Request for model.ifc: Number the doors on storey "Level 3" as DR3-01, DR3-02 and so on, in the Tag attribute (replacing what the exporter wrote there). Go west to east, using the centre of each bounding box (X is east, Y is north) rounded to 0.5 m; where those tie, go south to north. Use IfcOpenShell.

First a look at what the model holds.

```python
import ifcopenshell
import ifcopenshell.util.element
import ifcopenshell.util.placement

model = ifcopenshell.open("model.ifc")
print(model.schema)
storey = next(s for s in model.by_type("IfcBuildingStorey") if s.Name == "Level 3")
doors = [e for e in ifcopenshell.util.element.get_decomposition(storey) if e.is_a("IfcDoor")]
for e in sorted(doors, key=lambda e: e.id()):
    origin = ifcopenshell.util.placement.get_local_placement(e.ObjectPlacement)[:3, 3]
    print(e.id(), e.Tag, e.Name, origin.round(2) + 0.0, sep=" | ")
```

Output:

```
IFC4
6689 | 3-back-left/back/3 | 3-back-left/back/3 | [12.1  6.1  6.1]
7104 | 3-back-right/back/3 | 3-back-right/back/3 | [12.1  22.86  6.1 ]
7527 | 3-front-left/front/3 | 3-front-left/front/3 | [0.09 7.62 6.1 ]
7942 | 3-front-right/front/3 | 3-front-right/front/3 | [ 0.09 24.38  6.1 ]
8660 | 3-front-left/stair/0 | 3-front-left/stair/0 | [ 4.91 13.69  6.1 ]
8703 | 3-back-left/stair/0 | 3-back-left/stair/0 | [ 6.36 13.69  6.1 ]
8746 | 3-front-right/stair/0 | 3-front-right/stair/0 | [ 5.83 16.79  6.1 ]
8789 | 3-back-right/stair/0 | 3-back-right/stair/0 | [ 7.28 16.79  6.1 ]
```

```python
import ifcopenshell
import ifcopenshell.geom
import ifcopenshell.util.element
import ifcopenshell.util.shape

model = ifcopenshell.open("model.ifc")
settings = ifcopenshell.geom.settings()
settings.set("use-world-coords", True)


def centre(element):
    shape = ifcopenshell.geom.create_shape(settings, element)
    return ifcopenshell.util.shape.get_bbox_centroid(shape.geometry)


storey = next(s for s in model.by_type("IfcBuildingStorey") if s.Name == "Level 3")
doors = [e for e in ifcopenshell.util.element.get_decomposition(storey) if e.is_a("IfcDoor")]

# Insertion points can sit at a corner or the storey origin, so sort by the geometry (in metres).
centres = {e: centre(e) for e in doors}
doors.sort(key=lambda e: (round(centres[e][0] / 0.5), centres[e][1]))

for i, e in enumerate(doors, start=1):
    number = f"DR3-{i:02d}"
    e.Tag = number
    print(e.id(), number)

model.write("model_v2.ifc")
```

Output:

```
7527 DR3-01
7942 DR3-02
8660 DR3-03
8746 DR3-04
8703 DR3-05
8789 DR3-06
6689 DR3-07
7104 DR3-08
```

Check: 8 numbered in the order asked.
